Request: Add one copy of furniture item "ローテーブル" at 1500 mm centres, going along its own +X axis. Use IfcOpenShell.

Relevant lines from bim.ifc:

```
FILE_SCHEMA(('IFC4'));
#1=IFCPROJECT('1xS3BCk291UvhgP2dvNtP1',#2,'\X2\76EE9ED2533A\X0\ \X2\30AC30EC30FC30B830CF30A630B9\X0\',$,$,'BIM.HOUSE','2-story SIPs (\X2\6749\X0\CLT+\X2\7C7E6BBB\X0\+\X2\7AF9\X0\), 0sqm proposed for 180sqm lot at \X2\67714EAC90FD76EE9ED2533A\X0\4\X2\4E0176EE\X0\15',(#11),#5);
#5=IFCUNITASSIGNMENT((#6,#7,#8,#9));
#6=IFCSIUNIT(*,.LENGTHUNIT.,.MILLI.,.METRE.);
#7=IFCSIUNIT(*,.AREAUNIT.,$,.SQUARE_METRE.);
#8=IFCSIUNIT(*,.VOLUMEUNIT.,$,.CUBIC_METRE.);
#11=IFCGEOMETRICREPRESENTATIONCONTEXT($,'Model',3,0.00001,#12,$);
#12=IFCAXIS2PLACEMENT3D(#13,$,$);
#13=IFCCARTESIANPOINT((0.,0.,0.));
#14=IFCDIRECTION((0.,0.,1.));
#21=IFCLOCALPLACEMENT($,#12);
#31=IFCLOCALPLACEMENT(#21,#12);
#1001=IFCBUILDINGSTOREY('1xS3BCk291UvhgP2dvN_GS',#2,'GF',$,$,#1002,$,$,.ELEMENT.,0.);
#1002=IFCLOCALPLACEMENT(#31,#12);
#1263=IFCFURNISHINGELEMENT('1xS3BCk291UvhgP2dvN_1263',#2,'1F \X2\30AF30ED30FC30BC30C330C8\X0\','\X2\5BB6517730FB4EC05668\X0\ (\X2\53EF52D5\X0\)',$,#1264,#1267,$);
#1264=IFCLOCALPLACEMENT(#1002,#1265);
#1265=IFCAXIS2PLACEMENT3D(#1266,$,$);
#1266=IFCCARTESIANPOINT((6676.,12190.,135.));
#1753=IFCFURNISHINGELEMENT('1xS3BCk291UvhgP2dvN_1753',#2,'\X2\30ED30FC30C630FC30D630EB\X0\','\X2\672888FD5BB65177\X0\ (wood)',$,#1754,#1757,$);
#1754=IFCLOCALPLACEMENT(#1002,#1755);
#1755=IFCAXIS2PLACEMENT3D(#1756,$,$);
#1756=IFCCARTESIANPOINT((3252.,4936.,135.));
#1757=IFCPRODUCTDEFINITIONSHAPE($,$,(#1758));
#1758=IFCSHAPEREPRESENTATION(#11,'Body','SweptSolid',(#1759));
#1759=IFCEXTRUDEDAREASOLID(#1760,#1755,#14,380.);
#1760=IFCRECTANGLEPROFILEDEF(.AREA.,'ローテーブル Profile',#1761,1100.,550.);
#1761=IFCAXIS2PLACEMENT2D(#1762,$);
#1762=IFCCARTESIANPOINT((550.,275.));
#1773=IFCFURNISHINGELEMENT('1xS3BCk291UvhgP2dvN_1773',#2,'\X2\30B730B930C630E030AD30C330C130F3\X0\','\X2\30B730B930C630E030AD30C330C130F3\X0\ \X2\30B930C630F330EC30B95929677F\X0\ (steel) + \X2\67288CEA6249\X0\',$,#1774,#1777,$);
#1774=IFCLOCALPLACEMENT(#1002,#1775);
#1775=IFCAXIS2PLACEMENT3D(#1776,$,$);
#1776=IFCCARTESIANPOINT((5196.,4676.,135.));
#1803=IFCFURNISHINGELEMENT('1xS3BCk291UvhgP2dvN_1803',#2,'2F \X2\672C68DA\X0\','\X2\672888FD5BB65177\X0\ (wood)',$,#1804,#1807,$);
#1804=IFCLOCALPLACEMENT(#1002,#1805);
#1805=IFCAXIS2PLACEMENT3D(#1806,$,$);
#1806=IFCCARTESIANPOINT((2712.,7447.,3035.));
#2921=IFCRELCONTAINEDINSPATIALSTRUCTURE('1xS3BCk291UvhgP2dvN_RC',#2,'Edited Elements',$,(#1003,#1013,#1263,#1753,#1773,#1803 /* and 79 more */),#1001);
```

```python
import ifcopenshell
import ifcopenshell.api.geometry
import ifcopenshell.api.root
import ifcopenshell.util.element
import ifcopenshell.util.placement

model = ifcopenshell.open("bim.ifc")


def reuse_history(source, copy):
    """copy_class also copies each property set's owner history, people and application; keep the originals."""
    for rel in copy.IsDefinedBy:
        if rel.is_a("IfcRelDefinesByProperties") and (history := rel.RelatingPropertyDefinition.OwnerHistory):
            rel.RelatingPropertyDefinition.OwnerHistory = source.OwnerHistory
            ifcopenshell.util.element.remove_deep2(model, history)


source = model.by_guid("1xS3BCk291UvhgP2dvN_1753")
base = ifcopenshell.util.placement.get_local_placement(source.ObjectPlacement)
step = base[:3, 0] * 1500.0

for i in range(1, 2):
    copy = ifcopenshell.api.root.copy_class(model, product=source)
    copy.Representation = ifcopenshell.util.element.copy_deep(
        model, source.Representation, exclude=["IfcGeometricRepresentationContext", "IfcRepresentationMap"]
    )
    reuse_history(source, copy)
    matrix = base.copy()
    matrix[:3, 3] += i * step
    print("added at", matrix[:3, 3].round(3) + 0.0)
    ifcopenshell.api.geometry.edit_object_placement(model, product=copy, matrix=matrix, is_si=False)

model.write("bim-out.ifc")
```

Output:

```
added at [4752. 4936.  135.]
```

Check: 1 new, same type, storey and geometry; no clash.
